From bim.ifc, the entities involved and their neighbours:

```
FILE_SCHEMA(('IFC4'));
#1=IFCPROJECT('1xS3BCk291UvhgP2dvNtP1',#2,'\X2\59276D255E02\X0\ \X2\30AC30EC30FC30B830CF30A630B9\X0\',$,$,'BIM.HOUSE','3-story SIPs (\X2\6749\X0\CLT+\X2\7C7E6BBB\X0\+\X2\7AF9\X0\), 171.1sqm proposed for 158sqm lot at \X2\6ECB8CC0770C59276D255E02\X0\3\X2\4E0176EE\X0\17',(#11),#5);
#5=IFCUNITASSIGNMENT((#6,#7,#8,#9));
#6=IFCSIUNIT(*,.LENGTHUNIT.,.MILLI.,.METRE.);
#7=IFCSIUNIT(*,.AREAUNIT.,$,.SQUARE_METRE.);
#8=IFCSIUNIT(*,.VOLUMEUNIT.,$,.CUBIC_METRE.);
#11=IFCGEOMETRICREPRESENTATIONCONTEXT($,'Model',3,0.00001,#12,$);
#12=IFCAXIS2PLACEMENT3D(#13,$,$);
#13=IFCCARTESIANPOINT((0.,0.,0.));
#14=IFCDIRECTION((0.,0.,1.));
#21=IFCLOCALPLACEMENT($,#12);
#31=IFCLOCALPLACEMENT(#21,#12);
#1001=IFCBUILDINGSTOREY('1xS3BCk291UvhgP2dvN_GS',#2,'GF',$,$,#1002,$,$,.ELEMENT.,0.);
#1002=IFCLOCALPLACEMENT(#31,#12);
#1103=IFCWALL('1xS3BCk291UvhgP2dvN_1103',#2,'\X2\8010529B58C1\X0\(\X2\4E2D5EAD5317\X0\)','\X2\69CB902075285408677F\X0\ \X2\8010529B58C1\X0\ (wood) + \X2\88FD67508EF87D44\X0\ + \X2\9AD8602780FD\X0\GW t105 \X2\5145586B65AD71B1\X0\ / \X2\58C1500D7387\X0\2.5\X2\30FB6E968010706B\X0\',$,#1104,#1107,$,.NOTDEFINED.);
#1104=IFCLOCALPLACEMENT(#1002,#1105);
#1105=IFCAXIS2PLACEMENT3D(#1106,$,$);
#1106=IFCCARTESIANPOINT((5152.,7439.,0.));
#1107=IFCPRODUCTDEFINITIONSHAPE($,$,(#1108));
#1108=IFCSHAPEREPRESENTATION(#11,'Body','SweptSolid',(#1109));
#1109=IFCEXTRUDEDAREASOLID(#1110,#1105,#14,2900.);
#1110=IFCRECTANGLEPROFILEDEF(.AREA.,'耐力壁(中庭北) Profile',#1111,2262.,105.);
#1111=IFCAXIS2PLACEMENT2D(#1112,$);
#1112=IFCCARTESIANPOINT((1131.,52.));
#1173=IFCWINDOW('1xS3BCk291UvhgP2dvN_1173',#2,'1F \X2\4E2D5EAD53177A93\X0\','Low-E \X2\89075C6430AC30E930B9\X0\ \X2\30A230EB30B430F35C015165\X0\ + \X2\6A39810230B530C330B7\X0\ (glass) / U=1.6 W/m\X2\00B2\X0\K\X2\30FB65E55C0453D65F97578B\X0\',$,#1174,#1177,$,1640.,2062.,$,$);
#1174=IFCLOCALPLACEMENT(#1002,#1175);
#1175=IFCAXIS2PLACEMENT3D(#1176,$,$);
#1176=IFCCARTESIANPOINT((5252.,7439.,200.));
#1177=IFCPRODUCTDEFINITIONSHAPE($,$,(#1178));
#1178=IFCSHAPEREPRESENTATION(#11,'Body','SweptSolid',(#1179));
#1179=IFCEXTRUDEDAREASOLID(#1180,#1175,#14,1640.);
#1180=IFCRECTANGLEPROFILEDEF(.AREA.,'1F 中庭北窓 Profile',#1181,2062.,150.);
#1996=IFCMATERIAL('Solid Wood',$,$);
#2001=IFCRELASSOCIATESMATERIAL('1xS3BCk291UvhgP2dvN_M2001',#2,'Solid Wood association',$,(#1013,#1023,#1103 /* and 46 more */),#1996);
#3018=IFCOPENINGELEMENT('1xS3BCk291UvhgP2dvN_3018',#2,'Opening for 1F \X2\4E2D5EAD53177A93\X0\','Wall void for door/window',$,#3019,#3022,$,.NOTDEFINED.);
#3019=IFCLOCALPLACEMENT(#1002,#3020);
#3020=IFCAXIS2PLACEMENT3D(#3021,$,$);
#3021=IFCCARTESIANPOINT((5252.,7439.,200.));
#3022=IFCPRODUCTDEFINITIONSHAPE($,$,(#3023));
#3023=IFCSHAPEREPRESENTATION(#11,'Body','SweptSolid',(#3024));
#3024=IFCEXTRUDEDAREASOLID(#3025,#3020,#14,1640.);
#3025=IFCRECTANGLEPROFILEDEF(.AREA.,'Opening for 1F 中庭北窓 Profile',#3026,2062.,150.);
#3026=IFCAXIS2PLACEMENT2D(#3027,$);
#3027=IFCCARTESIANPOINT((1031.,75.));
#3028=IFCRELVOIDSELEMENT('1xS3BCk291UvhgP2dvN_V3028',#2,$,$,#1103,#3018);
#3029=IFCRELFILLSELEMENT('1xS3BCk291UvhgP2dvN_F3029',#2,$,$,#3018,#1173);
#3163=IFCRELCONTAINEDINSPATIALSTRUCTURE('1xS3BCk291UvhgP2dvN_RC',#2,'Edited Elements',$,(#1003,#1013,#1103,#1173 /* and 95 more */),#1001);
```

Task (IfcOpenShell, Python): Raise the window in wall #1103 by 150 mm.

```python
import numpy as np
import ifcopenshell
import ifcopenshell.api.geometry
import ifcopenshell.util.placement
import ifcopenshell.util.unit

model = ifcopenshell.open("bim.ifc")
unit_scale = ifcopenshell.util.unit.calculate_unit_scale(model)

window = model.by_guid("1xS3BCk291UvhgP2dvN_1173")
opening = window.FillsVoids[0].RelatingOpeningElement
dz = 0.15 / unit_scale

shift = np.array([0.0, 0.0, dz])
# The window is not placed relative to its opening, so move both.
for product in (opening, window):
    matrix = ifcopenshell.util.placement.get_local_placement(product.ObjectPlacement)
    matrix[:3, 3] += shift
    ifcopenshell.api.geometry.edit_object_placement(model, product=product, matrix=matrix, is_si=False)

print(f"moved by {dz * unit_scale:+.3f} m")

model.write("bim_edited.ifc")
```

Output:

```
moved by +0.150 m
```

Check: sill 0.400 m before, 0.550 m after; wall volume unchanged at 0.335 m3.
